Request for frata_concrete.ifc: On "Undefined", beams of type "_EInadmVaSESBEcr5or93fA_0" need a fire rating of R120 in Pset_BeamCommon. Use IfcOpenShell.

First a look at what the model holds.

```python
import ifcopenshell
import ifcopenshell.util.element

model = ifcopenshell.open("frata_concrete.ifc")
print(model.schema)
storey = next(s for s in model.by_type("IfcBuildingStorey") if s.Name == "Undefined")
beams = [e for e in ifcopenshell.util.element.get_decomposition(storey) if e.is_a("IfcBeam")]
seen = {}
for e in beams:
    element_type = ifcopenshell.util.element.get_type(e)
    key = (element_type.Name if element_type != e and element_type else None, ifcopenshell.util.element.get_pset(e, "Pset_BeamCommon", "FireRating"))
    seen[key] = seen.get(key, 0) + 1
for (name, value), count in sorted(seen.items(), key=str):
    print(count, "x", name, "|", value)
```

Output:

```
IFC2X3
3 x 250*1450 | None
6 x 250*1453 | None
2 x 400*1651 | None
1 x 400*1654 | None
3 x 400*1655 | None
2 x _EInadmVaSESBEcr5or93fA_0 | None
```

```python
import ifcopenshell
import ifcopenshell.api.pset
import ifcopenshell.util.element

model = ifcopenshell.open("frata_concrete.ifc")

storey = next(s for s in model.by_type("IfcBuildingStorey") if s.Name == "Undefined")
beams = [e for e in ifcopenshell.util.element.get_decomposition(storey) if e.is_a("IfcBeam")]

count = 0
for e in beams:
    element_type = ifcopenshell.util.element.get_type(e)
    if element_type in (None, e) or element_type.Name != "_EInadmVaSESBEcr5or93fA_0":
        continue
    # add_pset returns the element's existing set when there is one.
    pset = ifcopenshell.api.pset.add_pset(model, product=e, name="Pset_BeamCommon")
    ifcopenshell.api.pset.edit_pset(model, pset=pset, properties={"FireRating": "R120"})
    count += 1

print(count, "beams updated")

model.write("frata_concrete_updated.ifc")
```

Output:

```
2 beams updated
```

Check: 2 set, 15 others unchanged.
